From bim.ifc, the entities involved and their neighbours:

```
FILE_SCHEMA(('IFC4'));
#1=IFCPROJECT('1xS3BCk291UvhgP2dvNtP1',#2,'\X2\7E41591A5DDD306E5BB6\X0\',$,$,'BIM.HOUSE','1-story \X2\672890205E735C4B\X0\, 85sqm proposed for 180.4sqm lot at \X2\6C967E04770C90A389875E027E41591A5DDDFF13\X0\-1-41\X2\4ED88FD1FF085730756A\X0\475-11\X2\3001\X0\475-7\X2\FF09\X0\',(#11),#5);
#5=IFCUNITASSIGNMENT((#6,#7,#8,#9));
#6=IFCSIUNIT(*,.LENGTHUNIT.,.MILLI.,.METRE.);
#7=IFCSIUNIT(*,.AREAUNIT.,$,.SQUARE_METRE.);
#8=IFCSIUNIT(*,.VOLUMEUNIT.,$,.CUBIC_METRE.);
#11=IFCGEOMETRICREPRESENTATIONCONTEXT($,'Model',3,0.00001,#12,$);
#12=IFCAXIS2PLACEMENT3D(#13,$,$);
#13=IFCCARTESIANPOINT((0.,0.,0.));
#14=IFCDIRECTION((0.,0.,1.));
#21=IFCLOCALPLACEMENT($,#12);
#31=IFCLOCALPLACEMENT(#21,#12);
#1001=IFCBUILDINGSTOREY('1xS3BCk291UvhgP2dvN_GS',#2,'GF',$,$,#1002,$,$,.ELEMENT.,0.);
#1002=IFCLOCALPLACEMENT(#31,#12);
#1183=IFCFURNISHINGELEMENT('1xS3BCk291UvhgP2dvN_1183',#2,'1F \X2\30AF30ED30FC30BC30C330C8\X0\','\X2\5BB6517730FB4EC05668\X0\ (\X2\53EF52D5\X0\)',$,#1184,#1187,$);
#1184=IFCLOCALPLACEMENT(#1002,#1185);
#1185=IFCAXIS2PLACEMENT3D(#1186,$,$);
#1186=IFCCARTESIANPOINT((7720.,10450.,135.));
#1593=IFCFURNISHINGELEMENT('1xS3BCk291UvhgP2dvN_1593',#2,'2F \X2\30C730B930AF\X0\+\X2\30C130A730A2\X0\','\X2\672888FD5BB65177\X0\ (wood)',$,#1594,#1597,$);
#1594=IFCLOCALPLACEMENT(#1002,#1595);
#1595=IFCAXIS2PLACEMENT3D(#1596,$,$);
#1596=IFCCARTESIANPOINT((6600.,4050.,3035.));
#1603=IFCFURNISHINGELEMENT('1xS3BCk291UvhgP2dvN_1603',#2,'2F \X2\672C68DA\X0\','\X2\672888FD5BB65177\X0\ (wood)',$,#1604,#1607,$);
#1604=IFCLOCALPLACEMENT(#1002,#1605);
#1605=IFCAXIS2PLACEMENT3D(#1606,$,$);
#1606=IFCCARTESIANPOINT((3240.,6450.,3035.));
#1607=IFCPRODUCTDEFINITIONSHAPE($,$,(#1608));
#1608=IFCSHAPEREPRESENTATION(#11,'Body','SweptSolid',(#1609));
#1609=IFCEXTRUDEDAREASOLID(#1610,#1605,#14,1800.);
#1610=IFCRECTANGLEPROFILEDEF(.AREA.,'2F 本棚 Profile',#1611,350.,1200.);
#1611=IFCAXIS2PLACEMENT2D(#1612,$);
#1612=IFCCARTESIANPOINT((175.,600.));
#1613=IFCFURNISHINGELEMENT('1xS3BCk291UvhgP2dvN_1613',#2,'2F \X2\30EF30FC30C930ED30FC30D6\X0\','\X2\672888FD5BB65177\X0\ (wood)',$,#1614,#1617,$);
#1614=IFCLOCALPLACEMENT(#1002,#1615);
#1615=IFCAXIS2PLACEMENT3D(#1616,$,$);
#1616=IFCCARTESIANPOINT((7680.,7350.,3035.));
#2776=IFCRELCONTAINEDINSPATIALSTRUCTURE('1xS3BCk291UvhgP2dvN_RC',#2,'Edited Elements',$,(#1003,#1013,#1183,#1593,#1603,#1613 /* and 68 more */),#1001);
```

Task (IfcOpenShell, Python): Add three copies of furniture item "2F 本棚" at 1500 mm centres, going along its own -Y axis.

```python
import ifcopenshell
import ifcopenshell.api.geometry
import ifcopenshell.api.root
import ifcopenshell.util.element
import ifcopenshell.util.placement
import ifcopenshell.util.unit

model = ifcopenshell.open("bim.ifc")
unit_scale = ifcopenshell.util.unit.calculate_unit_scale(model)


def reuse_history(source, copy):
    """copy_class also copies each property set's owner history, people and application; keep the originals."""
    for rel in copy.IsDefinedBy:
        if rel.is_a("IfcRelDefinesByProperties") and (history := rel.RelatingPropertyDefinition.OwnerHistory):
            rel.RelatingPropertyDefinition.OwnerHistory = source.OwnerHistory
            ifcopenshell.util.element.remove_deep2(model, history)


source = model.by_guid("1xS3BCk291UvhgP2dvN_1603")
base = ifcopenshell.util.placement.get_local_placement(source.ObjectPlacement)
step = -base[:3, 1] * 1.5 / unit_scale

for i in range(1, 4):
    copy = ifcopenshell.api.root.copy_class(model, product=source)
    copy.Representation = ifcopenshell.util.element.copy_deep(
        model, source.Representation, exclude=["IfcGeometricRepresentationContext", "IfcRepresentationMap"]
    )
    reuse_history(source, copy)
    matrix = base.copy()
    matrix[:3, 3] += i * step
    print("added at", matrix[:3, 3].round(3) + 0.0)
    ifcopenshell.api.geometry.edit_object_placement(model, product=copy, matrix=matrix, is_si=False)

model.write("bim-out.ifc")
```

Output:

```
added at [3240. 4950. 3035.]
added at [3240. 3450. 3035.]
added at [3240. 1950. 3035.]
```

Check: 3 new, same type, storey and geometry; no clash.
